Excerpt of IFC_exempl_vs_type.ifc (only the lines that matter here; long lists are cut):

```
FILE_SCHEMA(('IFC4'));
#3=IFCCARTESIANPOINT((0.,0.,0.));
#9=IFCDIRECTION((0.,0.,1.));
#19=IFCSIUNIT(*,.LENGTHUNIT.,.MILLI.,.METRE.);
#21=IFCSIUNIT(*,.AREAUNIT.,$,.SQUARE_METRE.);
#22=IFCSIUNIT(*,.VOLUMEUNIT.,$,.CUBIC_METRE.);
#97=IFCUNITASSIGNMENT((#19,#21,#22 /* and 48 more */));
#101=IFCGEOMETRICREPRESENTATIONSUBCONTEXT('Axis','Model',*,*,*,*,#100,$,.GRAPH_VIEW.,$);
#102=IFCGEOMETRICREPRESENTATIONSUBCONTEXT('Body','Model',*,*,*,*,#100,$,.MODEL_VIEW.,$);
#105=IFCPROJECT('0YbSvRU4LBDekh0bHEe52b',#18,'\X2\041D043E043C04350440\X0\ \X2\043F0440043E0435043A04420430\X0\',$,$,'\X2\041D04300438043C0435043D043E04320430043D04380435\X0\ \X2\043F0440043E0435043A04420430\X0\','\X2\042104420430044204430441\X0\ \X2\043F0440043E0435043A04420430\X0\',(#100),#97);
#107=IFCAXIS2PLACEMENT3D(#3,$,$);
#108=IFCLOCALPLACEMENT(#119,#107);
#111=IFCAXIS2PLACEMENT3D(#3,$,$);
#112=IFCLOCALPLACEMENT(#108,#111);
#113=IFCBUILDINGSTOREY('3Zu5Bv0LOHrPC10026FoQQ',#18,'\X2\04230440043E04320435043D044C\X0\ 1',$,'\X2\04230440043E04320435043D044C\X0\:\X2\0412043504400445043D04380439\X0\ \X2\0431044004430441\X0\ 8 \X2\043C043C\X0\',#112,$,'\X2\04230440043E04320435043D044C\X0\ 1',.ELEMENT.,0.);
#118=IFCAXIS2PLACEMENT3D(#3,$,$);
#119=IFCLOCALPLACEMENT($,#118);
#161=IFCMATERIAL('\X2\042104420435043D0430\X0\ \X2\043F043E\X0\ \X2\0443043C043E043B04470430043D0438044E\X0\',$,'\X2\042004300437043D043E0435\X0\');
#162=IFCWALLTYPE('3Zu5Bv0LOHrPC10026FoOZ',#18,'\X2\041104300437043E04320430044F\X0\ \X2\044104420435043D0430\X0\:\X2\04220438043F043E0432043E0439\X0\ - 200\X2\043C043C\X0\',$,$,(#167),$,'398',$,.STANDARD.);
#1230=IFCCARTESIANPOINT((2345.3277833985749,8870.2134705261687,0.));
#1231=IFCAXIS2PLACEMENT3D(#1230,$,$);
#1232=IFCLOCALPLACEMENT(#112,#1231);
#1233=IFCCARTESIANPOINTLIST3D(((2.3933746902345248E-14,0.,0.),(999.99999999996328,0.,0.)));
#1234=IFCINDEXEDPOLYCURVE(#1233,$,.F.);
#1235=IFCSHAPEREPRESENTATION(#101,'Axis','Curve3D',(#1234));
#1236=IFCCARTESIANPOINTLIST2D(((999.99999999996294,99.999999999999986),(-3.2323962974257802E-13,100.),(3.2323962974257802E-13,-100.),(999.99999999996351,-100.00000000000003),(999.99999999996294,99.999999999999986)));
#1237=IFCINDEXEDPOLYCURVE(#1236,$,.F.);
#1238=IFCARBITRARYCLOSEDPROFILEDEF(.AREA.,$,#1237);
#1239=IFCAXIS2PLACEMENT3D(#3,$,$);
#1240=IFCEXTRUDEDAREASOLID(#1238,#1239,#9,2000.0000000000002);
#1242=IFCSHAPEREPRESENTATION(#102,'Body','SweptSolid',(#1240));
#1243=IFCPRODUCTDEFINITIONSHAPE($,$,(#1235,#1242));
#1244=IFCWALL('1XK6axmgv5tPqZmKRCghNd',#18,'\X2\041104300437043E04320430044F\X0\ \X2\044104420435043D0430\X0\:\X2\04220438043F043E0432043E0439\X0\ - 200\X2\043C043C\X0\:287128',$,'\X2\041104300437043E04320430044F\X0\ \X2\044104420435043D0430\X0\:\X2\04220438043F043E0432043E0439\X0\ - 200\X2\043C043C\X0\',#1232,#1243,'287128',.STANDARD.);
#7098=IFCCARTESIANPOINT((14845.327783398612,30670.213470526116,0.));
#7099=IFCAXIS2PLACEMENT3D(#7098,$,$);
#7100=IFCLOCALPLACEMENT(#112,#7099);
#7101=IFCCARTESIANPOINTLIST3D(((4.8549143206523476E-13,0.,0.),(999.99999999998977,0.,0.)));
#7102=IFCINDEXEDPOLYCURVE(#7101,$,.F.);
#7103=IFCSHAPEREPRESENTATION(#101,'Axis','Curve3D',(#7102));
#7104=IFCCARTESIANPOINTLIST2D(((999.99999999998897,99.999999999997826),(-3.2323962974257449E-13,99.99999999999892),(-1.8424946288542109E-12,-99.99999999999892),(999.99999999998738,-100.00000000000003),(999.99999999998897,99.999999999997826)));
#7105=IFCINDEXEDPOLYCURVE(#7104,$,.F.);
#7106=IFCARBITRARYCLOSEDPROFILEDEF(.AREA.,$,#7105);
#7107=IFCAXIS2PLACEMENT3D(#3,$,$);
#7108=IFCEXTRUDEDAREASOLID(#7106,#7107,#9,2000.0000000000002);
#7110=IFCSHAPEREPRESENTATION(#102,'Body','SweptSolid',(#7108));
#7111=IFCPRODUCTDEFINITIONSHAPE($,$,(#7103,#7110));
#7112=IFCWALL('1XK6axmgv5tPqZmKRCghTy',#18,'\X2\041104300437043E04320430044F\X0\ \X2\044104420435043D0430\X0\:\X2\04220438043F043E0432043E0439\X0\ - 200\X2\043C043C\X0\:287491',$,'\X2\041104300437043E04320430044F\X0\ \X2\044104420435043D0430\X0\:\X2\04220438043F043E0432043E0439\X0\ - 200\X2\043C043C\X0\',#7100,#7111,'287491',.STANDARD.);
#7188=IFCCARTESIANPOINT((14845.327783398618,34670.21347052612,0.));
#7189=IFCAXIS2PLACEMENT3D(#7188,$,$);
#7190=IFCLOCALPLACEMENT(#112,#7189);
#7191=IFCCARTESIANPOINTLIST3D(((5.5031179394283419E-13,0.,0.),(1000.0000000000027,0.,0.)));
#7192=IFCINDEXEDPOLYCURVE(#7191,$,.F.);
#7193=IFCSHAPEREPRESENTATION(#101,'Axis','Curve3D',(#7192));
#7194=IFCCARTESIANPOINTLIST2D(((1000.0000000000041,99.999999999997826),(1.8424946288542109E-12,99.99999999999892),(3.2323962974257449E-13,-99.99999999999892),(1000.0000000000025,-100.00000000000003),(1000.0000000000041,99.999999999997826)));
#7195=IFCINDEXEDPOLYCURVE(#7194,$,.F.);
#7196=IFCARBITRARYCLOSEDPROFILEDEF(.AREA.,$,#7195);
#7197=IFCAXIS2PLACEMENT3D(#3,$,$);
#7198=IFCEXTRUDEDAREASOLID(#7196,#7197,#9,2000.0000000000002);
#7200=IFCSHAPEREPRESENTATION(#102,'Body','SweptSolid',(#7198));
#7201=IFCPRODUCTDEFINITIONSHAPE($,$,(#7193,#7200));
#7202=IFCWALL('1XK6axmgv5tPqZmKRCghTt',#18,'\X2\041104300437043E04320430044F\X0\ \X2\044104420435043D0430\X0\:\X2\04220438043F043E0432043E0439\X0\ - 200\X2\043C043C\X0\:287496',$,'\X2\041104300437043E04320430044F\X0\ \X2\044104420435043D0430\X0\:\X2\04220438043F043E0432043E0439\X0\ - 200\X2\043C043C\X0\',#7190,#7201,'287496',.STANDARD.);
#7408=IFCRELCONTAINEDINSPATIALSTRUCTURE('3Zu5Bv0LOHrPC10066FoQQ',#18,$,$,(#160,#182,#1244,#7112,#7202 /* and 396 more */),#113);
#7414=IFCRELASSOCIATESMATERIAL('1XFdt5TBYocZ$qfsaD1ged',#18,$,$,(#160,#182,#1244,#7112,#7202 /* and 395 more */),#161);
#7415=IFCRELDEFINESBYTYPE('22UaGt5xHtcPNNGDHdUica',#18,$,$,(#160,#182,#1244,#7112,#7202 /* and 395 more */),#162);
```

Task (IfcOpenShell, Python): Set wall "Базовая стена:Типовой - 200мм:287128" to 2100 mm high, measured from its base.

```python
import ifcopenshell
import ifcopenshell.geom
import ifcopenshell.util.representation
import ifcopenshell.util.shape

model = ifcopenshell.open("IFC_exempl_vs_type.ifc")
settings = ifcopenshell.geom.settings()


def volume(element):
    """Net volume in cubic metres, openings subtracted."""
    shape = ifcopenshell.geom.create_shape(settings, element)
    return ifcopenshell.util.shape.get_volume(shape.geometry)


wall = model.by_id(1244)
before = volume(wall)

body = ifcopenshell.util.representation.get_representation(wall, "Model", "Body")
solid = body.Items[0]
old_height = solid.Depth
solid.Depth = 2100.0
after = volume(wall)

print(f"height {old_height:g} -> {solid.Depth:g}, volume {before:.3f} -> {after:.3f} m3")

model.write("IFC_exempl_vs_type-out.ifc")
```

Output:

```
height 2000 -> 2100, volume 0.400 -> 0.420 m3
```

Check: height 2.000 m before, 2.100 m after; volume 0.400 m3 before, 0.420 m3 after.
